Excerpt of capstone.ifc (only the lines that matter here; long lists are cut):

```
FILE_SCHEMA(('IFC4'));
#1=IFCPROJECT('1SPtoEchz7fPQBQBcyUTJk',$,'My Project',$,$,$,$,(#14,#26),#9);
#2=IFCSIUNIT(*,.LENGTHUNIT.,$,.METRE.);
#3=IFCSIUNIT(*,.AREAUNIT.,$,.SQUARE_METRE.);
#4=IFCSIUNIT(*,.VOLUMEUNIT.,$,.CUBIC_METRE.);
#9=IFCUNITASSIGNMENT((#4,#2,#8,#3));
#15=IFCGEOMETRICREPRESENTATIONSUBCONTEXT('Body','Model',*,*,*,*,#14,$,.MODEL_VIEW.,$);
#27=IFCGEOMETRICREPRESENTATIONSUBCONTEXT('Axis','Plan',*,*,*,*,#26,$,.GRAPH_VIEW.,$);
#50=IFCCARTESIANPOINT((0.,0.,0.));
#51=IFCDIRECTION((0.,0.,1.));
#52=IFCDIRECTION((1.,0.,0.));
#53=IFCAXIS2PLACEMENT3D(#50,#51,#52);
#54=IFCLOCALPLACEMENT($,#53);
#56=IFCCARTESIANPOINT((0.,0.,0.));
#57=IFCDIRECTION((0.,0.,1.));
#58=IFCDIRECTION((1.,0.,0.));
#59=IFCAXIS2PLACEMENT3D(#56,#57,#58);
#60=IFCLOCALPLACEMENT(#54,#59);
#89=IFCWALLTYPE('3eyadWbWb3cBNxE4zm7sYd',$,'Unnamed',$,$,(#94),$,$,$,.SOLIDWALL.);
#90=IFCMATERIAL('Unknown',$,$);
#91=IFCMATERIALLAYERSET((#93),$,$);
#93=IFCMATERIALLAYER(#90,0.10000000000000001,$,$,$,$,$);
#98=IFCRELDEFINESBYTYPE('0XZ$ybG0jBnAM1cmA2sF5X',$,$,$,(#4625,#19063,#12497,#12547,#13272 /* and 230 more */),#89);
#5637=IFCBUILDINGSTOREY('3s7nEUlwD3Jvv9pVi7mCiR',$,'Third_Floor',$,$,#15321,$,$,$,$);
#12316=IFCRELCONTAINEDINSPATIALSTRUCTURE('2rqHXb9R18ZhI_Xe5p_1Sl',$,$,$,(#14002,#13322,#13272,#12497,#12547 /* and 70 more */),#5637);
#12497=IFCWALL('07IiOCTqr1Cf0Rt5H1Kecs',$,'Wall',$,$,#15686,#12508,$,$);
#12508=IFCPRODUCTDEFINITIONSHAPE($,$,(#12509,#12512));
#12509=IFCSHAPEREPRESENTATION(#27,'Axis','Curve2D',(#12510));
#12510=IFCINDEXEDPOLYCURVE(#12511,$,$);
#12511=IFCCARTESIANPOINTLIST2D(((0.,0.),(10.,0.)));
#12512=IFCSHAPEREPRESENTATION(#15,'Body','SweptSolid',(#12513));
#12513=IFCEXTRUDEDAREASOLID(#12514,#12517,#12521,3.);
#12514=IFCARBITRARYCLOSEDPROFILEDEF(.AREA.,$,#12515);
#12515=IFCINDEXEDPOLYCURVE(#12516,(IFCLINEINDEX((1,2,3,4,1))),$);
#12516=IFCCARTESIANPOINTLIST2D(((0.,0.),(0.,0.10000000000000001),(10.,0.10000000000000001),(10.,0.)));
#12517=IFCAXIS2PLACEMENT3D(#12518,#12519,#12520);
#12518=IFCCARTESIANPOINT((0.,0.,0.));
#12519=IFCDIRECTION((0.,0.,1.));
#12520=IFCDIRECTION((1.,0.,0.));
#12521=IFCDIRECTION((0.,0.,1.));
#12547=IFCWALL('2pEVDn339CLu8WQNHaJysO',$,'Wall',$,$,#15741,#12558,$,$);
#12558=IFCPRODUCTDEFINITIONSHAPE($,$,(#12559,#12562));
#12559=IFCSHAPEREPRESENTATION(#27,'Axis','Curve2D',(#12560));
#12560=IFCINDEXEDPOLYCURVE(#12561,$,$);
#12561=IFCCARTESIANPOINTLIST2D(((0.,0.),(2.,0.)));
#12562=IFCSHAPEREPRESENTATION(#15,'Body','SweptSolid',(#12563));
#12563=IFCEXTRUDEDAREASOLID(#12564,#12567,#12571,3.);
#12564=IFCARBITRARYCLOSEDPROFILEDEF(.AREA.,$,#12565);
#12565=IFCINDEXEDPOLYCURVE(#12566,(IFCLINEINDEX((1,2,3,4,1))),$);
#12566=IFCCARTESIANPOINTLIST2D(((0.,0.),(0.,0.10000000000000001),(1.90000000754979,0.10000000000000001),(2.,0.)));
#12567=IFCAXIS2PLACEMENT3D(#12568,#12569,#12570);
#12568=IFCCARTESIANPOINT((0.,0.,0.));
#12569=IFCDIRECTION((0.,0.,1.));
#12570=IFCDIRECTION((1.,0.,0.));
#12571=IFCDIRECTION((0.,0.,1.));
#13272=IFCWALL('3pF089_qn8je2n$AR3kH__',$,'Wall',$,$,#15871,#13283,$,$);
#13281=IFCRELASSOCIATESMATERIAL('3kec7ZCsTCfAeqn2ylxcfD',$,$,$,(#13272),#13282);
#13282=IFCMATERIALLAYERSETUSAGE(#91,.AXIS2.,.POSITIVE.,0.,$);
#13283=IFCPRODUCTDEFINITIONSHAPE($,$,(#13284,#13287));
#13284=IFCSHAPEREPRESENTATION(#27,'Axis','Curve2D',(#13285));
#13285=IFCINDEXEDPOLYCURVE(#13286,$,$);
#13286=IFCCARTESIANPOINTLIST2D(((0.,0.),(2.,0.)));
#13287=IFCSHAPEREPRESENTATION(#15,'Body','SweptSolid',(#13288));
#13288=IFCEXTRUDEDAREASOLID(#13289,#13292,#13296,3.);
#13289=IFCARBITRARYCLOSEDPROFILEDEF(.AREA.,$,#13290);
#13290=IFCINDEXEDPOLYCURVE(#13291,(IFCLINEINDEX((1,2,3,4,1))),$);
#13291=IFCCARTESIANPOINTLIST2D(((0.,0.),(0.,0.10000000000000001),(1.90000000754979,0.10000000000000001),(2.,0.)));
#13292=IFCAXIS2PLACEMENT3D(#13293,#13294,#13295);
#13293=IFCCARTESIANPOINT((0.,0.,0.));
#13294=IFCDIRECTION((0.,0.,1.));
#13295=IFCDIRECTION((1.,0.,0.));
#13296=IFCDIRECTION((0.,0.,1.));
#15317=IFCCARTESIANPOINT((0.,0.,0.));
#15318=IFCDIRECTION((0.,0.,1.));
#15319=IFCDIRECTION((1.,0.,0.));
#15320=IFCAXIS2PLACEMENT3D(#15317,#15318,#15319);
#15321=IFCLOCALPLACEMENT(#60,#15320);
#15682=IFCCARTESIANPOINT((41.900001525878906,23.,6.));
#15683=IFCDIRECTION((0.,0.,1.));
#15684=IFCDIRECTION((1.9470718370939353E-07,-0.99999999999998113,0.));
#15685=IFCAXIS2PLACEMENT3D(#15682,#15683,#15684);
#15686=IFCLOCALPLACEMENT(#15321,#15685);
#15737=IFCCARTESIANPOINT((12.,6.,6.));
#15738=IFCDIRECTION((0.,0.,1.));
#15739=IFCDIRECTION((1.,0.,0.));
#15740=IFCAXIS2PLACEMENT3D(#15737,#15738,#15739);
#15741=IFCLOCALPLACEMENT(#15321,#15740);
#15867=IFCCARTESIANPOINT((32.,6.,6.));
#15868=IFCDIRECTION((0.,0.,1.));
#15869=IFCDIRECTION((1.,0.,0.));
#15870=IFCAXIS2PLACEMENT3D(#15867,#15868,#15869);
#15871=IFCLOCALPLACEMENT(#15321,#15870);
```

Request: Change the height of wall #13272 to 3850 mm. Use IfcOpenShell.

```python
import ifcopenshell
import ifcopenshell.geom
import ifcopenshell.util.representation
import ifcopenshell.util.shape

model = ifcopenshell.open("capstone.ifc")
settings = ifcopenshell.geom.settings()


def volume(element):
    """Net volume in cubic metres, openings subtracted."""
    shape = ifcopenshell.geom.create_shape(settings, element)
    return ifcopenshell.util.shape.get_volume(shape.geometry)


wall = model.by_guid("3pF089_qn8je2n$AR3kH__")
before = volume(wall)

body = ifcopenshell.util.representation.get_representation(wall, "Model", "Body")
solid = body.Items[0]
old_height = solid.Depth
solid.Depth = 3.85
after = volume(wall)

print(f"height {old_height:g} -> {solid.Depth:g}, volume {before:.3f} -> {after:.3f} m3")

model.write("capstone_edited.ifc")
```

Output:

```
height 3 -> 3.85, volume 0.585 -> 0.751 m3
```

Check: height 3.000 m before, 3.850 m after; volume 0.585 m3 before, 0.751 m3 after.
